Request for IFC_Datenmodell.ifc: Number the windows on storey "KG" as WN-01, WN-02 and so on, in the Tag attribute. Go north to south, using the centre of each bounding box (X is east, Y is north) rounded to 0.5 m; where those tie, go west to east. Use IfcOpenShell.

First a look at what the model holds.

```python
import ifcopenshell
import ifcopenshell.util.element
import ifcopenshell.util.placement

model = ifcopenshell.open("IFC_Datenmodell.ifc")
print(model.schema)
storey = next(s for s in model.by_type("IfcBuildingStorey") if s.Name == "KG")
windows = [e for e in ifcopenshell.util.element.get_decomposition(storey) if e.is_a("IfcWindow")]
for e in sorted(windows, key=lambda e: e.id()):
    origin = ifcopenshell.util.placement.get_local_placement(e.ObjectPlacement)[:3, 3]
    print(e.id(), e.Tag, e.Name, origin.round(2) + 0.0, sep=" | ")
```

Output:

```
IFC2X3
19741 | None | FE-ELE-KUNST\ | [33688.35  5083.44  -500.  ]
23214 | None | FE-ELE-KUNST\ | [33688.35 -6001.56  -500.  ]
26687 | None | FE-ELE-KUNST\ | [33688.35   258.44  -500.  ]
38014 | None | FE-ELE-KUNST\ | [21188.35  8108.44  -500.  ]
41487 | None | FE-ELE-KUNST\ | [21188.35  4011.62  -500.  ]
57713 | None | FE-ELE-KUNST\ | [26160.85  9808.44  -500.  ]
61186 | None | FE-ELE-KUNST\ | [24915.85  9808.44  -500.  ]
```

```python
import ifcopenshell
import ifcopenshell.geom
import ifcopenshell.util.element
import ifcopenshell.util.shape

model = ifcopenshell.open("IFC_Datenmodell.ifc")
settings = ifcopenshell.geom.settings()
settings.set("use-world-coords", True)


def centre(element):
    shape = ifcopenshell.geom.create_shape(settings, element)
    return ifcopenshell.util.shape.get_bbox_centroid(shape.geometry)


storey = next(s for s in model.by_type("IfcBuildingStorey") if s.Name == "KG")
windows = [e for e in ifcopenshell.util.element.get_decomposition(storey) if e.is_a("IfcWindow")]

# Insertion points can sit at a corner or the storey origin, so sort by the geometry (in metres).
centres = {e: centre(e) for e in windows}
windows.sort(key=lambda e: (-round(centres[e][1] / 0.5), centres[e][0]))

for i, e in enumerate(windows, start=1):
    number = f"WN-{i:02d}"
    e.Tag = number
    print(e.id(), number)

model.write("IFC_Datenmodell_rev.ifc")
```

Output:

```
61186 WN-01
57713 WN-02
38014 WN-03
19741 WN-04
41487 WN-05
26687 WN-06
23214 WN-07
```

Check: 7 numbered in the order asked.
